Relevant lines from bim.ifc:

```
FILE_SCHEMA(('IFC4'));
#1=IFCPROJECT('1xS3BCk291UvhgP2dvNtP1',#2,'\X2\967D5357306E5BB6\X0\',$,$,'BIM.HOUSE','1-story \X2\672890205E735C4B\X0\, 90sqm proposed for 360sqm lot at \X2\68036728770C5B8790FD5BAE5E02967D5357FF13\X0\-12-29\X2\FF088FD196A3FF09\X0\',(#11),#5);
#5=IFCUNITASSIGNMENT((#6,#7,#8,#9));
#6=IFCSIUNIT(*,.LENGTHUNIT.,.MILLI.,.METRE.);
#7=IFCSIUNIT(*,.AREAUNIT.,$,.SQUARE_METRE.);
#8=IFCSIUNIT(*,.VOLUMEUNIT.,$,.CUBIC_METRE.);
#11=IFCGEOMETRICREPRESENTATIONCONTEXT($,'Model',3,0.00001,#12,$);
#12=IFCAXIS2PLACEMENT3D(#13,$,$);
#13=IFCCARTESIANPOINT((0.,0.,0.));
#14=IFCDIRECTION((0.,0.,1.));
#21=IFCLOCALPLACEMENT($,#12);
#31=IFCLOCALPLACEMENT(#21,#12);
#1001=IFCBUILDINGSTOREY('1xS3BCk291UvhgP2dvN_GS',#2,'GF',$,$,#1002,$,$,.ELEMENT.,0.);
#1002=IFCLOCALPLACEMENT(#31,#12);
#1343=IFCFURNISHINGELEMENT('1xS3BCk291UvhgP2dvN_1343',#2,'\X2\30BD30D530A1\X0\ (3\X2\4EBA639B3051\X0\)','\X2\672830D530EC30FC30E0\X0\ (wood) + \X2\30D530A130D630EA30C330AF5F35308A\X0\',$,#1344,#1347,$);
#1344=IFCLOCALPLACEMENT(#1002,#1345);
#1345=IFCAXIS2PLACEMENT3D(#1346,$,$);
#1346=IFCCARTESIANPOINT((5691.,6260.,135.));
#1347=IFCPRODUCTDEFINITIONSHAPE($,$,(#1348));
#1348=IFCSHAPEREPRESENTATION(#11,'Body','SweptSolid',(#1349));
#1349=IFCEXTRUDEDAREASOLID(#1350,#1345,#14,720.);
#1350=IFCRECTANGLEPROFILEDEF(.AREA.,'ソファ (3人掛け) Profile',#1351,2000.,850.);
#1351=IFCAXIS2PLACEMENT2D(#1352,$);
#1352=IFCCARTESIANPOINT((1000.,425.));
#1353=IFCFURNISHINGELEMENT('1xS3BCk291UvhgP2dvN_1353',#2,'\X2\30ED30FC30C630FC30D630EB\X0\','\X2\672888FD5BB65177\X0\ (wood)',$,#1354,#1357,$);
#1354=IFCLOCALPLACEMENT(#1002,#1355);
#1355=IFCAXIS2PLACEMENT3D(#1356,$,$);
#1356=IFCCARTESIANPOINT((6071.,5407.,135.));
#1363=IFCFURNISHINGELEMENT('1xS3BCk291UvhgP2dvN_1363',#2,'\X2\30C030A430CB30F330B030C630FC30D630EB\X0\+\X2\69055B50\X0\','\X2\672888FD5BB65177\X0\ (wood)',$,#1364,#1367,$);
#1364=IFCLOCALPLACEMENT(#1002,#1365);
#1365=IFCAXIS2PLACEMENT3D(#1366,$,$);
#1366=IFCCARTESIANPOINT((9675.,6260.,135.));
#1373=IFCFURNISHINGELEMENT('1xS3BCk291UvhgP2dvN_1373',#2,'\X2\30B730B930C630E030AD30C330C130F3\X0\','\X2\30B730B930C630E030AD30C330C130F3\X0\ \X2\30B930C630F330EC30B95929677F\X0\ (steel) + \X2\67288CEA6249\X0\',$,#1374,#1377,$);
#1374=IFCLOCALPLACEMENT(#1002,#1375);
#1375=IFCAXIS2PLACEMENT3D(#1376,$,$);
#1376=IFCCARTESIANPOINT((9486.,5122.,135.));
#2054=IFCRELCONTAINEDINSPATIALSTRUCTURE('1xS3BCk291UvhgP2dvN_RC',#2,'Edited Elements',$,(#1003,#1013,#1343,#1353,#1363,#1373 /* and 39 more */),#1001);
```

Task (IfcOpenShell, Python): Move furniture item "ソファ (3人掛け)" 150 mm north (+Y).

```python
import ifcopenshell
import ifcopenshell.api.geometry
import ifcopenshell.util.placement

model = ifcopenshell.open("bim.ifc")

item = model.by_guid("1xS3BCk291UvhgP2dvN_1343")
matrix = ifcopenshell.util.placement.get_local_placement(item.ObjectPlacement)
matrix[1, 3] += 150.0
ifcopenshell.api.geometry.edit_object_placement(model, product=item, matrix=matrix, is_si=False)

print(ifcopenshell.util.placement.get_local_placement(item.ObjectPlacement).round(3) + 0.0)

model.write("bim-out.ifc")
```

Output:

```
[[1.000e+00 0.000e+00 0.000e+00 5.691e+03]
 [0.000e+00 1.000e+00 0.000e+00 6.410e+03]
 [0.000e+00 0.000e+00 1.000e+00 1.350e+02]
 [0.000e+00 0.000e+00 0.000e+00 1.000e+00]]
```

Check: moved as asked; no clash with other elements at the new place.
